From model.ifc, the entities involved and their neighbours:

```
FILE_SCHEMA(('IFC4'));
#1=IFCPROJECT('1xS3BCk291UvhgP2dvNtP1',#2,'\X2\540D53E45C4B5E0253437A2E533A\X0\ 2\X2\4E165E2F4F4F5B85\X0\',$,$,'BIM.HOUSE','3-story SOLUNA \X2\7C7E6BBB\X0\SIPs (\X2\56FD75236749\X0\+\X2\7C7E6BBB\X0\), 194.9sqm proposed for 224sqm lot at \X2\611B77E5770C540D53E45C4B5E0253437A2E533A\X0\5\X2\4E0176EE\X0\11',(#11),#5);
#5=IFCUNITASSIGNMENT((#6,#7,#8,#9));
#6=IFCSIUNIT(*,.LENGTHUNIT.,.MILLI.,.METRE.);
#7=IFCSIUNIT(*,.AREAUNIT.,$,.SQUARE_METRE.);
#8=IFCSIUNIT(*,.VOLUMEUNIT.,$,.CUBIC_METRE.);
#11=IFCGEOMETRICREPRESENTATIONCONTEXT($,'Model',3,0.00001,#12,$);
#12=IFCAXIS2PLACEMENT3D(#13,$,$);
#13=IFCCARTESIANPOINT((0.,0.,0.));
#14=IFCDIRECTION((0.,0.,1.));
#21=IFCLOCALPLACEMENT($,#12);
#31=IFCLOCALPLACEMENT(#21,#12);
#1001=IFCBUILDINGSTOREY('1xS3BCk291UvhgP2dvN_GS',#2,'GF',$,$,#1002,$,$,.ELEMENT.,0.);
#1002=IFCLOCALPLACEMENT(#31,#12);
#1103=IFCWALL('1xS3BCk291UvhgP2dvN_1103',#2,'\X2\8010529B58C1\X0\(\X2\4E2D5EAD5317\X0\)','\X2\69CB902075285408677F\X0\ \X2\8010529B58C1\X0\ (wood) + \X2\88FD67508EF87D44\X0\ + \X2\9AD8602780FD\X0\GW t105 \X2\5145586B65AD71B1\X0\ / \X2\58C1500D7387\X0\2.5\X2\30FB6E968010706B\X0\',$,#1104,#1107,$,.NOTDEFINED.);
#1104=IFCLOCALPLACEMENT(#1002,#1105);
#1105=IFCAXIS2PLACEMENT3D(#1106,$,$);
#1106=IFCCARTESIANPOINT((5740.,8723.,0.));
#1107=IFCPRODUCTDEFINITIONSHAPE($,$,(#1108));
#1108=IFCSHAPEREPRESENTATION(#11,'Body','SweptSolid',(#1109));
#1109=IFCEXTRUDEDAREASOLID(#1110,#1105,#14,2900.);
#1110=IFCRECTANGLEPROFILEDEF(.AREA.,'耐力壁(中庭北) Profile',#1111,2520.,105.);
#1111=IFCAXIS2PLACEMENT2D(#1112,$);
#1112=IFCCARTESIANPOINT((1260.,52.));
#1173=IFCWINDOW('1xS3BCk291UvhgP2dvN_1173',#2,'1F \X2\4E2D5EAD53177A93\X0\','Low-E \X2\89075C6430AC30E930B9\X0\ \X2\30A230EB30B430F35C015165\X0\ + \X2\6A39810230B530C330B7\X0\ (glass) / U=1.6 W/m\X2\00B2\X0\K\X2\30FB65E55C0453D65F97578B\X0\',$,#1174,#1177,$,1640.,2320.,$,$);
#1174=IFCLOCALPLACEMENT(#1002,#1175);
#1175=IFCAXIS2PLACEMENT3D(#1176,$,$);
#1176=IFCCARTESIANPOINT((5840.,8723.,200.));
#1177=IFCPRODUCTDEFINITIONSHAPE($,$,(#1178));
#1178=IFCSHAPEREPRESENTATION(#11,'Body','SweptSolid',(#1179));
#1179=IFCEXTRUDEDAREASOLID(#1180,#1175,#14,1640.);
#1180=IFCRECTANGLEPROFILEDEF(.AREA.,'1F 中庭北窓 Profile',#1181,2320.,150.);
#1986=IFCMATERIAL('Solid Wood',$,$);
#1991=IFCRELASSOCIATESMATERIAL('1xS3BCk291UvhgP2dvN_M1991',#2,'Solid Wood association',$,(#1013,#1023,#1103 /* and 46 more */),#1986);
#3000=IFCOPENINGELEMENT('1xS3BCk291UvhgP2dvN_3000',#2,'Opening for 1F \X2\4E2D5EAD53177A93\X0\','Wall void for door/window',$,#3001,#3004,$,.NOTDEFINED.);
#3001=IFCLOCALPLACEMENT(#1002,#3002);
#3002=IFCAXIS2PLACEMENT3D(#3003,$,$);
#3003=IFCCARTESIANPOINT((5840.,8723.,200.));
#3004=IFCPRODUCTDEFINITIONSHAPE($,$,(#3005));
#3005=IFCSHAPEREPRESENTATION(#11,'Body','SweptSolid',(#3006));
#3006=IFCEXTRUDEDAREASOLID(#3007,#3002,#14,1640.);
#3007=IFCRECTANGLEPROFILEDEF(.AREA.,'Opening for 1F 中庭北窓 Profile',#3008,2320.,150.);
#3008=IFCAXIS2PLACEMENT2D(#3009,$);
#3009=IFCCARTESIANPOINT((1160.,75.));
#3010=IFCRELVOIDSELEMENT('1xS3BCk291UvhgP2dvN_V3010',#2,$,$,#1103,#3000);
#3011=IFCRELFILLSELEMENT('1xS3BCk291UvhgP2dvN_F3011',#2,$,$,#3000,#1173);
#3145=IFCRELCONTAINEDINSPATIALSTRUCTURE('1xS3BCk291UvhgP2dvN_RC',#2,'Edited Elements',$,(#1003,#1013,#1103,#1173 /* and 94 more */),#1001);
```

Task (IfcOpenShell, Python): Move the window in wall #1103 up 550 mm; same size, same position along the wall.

```python
import numpy as np
import ifcopenshell
import ifcopenshell.api.geometry
import ifcopenshell.util.placement
import ifcopenshell.util.unit

model = ifcopenshell.open("model.ifc")
unit_scale = ifcopenshell.util.unit.calculate_unit_scale(model)

window = model.by_guid("1xS3BCk291UvhgP2dvN_1173")
opening = window.FillsVoids[0].RelatingOpeningElement
dz = 550.0

shift = np.array([0.0, 0.0, dz])
# The window is not placed relative to its opening, so move both.
for product in (opening, window):
    matrix = ifcopenshell.util.placement.get_local_placement(product.ObjectPlacement)
    matrix[:3, 3] += shift
    ifcopenshell.api.geometry.edit_object_placement(model, product=product, matrix=matrix, is_si=False)

print(f"moved by {dz * unit_scale:+.3f} m")

model.write("model_updated.ifc")
```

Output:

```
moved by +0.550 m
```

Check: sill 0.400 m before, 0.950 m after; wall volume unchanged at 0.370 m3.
